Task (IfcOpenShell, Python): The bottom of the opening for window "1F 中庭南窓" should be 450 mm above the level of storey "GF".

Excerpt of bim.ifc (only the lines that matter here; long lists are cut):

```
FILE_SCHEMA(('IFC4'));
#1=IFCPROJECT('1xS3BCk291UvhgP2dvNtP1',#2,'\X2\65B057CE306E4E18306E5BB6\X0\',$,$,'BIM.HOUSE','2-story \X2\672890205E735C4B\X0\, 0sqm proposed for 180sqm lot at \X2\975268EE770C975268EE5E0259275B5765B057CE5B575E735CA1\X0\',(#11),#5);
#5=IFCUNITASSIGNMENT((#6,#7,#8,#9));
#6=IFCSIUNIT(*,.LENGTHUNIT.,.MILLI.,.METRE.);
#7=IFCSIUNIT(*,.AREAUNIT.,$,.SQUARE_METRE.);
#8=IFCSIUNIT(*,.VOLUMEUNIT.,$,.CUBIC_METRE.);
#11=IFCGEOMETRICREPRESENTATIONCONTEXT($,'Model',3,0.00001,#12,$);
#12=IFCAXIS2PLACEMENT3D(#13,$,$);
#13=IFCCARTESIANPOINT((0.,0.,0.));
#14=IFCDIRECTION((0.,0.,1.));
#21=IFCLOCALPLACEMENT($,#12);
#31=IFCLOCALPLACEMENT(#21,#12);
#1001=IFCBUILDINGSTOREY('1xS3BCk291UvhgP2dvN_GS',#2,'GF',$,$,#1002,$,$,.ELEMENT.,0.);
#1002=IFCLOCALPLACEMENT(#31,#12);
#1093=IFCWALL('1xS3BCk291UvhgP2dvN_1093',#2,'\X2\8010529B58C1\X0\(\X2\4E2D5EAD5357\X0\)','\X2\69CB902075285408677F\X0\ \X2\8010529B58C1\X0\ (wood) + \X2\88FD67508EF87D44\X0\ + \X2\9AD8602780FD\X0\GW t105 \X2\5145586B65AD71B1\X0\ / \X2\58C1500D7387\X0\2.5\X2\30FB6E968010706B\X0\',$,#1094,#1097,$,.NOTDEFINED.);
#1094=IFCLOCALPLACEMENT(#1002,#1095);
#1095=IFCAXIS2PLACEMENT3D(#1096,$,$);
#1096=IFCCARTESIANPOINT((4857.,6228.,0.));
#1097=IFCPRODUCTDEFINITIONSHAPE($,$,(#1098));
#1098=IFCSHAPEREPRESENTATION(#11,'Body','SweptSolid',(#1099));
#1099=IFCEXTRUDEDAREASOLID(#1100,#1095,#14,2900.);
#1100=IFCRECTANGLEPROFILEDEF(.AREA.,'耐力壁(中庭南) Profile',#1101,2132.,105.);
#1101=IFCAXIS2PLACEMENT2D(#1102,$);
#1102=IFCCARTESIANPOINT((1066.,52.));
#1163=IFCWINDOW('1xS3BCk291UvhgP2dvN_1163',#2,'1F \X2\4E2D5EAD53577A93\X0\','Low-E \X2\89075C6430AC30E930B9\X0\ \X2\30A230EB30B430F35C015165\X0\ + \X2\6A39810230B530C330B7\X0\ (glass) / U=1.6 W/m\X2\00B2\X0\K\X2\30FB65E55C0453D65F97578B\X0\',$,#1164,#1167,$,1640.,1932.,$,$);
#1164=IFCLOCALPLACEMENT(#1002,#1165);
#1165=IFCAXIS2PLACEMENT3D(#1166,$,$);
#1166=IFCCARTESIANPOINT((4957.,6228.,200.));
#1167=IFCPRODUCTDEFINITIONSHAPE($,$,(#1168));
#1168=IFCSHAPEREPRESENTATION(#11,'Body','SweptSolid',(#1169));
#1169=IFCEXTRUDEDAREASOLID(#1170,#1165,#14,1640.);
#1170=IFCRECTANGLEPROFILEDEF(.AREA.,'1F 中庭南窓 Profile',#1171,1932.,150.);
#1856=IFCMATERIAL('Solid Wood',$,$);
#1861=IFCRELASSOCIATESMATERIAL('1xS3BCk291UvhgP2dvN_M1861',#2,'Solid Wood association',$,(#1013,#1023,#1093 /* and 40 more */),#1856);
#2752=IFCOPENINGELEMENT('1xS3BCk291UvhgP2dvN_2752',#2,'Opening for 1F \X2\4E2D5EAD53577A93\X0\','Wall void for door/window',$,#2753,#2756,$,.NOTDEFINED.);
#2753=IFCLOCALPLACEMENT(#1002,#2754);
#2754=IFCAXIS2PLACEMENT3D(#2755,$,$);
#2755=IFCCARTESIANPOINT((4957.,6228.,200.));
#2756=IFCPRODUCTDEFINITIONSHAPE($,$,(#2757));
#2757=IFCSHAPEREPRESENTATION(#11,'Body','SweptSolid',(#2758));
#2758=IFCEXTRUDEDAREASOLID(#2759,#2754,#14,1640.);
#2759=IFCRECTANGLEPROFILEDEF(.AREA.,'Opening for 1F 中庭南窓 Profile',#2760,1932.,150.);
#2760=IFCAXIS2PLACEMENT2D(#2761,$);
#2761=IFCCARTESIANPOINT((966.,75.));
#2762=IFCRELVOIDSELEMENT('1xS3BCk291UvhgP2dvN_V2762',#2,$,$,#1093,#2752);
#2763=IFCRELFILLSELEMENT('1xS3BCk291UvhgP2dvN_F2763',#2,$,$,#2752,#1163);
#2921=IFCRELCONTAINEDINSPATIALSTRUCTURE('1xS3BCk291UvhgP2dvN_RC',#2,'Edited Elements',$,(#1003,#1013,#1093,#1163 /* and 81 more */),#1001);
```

```python
import numpy as np
import ifcopenshell
import ifcopenshell.api.geometry
import ifcopenshell.geom
import ifcopenshell.util.element
import ifcopenshell.util.placement
import ifcopenshell.util.shape
import ifcopenshell.util.unit

model = ifcopenshell.open("bim.ifc")
unit_scale = ifcopenshell.util.unit.calculate_unit_scale(model)

window = model.by_id(1163)
opening = window.FillsVoids[0].RelatingOpeningElement
storey = ifcopenshell.util.element.get_container(window, ifc_class="IfcBuildingStorey")
level = ifcopenshell.util.placement.get_local_placement(storey.ObjectPlacement)[2, 3]

# The opening's origin need not be at the sill, so measure its lowest point.
shape = ifcopenshell.geom.create_shape(ifcopenshell.geom.settings(), opening)
bottom = ifcopenshell.util.shape.get_shape_bottom_elevation(shape, shape.geometry) / unit_scale
dz = level + 0.45 / unit_scale - bottom

shift = np.array([0.0, 0.0, dz])
# The window is not placed relative to its opening, so move both.
for product in (opening, window):
    matrix = ifcopenshell.util.placement.get_local_placement(product.ObjectPlacement)
    matrix[:3, 3] += shift
    ifcopenshell.api.geometry.edit_object_placement(model, product=product, matrix=matrix, is_si=False)

print(f"moved by {dz * unit_scale:+.3f} m")

model.write("bim_v2.ifc")
```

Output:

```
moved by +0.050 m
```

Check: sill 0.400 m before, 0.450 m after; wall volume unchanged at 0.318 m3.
